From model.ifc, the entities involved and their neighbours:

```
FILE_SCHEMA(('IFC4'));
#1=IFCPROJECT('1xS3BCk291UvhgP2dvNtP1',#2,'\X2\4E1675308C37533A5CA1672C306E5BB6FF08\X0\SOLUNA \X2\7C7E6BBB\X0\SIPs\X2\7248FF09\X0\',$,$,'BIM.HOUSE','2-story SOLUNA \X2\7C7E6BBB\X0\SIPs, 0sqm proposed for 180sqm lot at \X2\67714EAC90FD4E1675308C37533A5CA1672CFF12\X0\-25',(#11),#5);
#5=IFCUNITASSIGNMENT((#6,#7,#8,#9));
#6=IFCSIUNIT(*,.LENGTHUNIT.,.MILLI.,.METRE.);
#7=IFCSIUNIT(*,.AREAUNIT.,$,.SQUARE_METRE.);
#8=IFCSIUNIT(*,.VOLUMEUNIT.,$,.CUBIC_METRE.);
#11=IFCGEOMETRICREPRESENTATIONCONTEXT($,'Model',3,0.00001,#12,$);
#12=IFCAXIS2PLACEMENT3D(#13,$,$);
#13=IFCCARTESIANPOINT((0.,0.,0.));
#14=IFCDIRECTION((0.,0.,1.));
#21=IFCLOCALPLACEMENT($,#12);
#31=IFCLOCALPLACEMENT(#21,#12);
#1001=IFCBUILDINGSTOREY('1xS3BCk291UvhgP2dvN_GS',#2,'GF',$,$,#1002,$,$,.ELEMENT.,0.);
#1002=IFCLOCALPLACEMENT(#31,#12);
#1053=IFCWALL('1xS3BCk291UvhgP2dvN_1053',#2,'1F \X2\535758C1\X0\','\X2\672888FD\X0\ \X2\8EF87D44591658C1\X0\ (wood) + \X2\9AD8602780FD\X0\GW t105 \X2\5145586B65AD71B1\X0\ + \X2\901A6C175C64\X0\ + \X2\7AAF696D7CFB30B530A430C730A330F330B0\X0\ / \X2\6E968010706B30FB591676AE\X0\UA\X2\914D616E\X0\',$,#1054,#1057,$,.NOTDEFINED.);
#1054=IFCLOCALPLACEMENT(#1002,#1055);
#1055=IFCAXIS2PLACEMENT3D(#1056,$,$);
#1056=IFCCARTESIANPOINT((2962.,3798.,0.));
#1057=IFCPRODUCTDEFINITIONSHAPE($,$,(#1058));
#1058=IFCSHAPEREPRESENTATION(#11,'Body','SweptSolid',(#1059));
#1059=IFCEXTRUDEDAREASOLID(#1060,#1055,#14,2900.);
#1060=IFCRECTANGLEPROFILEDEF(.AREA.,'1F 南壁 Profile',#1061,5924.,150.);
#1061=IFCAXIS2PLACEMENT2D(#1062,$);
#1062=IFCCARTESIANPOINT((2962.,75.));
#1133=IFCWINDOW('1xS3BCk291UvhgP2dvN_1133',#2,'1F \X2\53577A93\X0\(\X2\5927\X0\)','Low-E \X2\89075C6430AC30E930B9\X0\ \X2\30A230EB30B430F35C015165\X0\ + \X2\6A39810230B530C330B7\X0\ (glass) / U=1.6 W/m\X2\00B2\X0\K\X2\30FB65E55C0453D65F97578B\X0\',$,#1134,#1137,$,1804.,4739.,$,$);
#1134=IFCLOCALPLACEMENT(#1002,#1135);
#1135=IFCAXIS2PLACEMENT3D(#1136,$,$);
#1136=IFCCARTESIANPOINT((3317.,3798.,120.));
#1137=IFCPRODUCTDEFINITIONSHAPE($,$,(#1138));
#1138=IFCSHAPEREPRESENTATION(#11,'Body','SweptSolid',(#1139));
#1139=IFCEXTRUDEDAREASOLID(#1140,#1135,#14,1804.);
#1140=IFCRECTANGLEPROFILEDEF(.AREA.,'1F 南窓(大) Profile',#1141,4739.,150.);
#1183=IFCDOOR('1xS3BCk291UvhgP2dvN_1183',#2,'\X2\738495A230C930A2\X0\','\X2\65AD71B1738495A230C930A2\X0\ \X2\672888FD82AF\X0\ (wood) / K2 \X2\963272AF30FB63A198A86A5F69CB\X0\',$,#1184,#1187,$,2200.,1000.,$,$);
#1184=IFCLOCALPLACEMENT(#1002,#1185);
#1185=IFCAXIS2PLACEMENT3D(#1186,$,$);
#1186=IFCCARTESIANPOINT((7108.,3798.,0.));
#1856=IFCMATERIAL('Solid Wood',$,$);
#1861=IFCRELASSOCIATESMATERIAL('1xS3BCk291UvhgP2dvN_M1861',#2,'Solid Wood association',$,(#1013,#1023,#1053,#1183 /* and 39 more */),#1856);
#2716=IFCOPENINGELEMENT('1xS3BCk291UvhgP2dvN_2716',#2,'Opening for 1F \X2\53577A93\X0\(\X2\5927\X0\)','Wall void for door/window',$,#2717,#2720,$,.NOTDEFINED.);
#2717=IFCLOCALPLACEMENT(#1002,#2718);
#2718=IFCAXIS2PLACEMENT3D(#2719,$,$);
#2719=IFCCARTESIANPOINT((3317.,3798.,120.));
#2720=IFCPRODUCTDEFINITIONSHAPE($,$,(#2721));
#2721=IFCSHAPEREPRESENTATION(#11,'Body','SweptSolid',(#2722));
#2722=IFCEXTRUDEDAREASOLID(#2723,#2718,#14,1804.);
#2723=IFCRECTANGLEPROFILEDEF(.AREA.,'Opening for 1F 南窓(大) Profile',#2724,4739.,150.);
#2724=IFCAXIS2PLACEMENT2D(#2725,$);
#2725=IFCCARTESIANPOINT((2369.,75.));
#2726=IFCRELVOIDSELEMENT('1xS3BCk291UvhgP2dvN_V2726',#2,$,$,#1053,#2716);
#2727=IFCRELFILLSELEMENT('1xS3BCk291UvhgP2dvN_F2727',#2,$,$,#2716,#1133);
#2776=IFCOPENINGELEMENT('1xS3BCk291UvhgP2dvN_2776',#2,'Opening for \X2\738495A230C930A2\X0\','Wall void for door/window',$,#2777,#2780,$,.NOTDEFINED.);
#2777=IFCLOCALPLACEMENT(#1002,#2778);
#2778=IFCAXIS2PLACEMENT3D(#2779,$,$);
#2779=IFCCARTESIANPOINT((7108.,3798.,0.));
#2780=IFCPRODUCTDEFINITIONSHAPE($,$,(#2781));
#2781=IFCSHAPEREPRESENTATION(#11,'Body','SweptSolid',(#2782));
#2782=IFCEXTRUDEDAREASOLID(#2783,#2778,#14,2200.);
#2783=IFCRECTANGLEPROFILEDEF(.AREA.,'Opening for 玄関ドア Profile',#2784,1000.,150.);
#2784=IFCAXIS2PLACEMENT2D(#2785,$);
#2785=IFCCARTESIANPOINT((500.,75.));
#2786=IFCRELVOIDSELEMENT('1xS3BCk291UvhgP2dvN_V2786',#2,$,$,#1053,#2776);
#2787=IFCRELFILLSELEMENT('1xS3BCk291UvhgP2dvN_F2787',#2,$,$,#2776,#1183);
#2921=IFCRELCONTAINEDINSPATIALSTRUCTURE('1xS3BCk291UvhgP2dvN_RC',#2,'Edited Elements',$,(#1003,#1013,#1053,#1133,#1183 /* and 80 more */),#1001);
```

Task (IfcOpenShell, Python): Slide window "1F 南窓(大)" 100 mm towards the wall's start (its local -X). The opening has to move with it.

```python
import ifcopenshell
import ifcopenshell.api.geometry
import ifcopenshell.util.placement

model = ifcopenshell.open("model.ifc")

window = model.by_guid("1xS3BCk291UvhgP2dvN_1133")
opening = window.FillsVoids[0].RelatingOpeningElement
wall = opening.VoidsElements[0].RelatingBuildingElement

wall_matrix = ifcopenshell.util.placement.get_local_placement(wall.ObjectPlacement)
shift = wall_matrix[:3, 0] * -100.0
before = ifcopenshell.util.placement.get_local_placement(window.ObjectPlacement)[:3, 3].copy()

# The window is not placed relative to its opening, so move both.
for product in (opening, window):
    matrix = ifcopenshell.util.placement.get_local_placement(product.ObjectPlacement)
    matrix[:3, 3] += shift
    ifcopenshell.api.geometry.edit_object_placement(model, product=product, matrix=matrix, is_si=False)

after = ifcopenshell.util.placement.get_local_placement(window.ObjectPlacement)[:3, 3]
print("window moved by", (after - before).round(3) + 0.0)

model.write("model_rev.ifc")
```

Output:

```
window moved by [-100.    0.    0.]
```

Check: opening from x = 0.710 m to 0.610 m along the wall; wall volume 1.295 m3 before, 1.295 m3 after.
